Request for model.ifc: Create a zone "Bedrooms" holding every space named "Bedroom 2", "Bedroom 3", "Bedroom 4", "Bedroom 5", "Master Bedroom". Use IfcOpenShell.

First a look at what the model holds.

```python
import ifcopenshell

model = ifcopenshell.open("model.ifc")
print(model.schema)
seen = {}
for space in model.by_type("IfcSpace"):
    seen[space.LongName] = seen.get(space.LongName, 0) + 1
for name, count in sorted(seen.items(), key=str):
    print(count, "x", name)
print("zones:", [z.Name for z in model.by_type("IfcZone")][:20])
```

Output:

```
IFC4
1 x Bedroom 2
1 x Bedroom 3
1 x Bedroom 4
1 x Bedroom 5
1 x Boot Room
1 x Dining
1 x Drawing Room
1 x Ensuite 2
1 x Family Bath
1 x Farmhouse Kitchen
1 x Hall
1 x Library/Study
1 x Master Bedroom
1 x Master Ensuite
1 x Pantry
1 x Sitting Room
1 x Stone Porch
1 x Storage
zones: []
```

```python
import ifcopenshell
import ifcopenshell.api.group
import ifcopenshell.api.root

model = ifcopenshell.open("model.ifc")

names = {"Bedroom 2", "Bedroom 3", "Bedroom 4", "Bedroom 5", "Master Bedroom"}
spaces = [s for s in model.by_type("IfcSpace") if s.LongName in names]

zone = ifcopenshell.api.root.create_entity(model, ifc_class="IfcZone", name="Bedrooms")
ifcopenshell.api.group.assign_group(model, products=spaces, group=zone)
print(len(spaces), "spaces in", zone.Name)

model.write("model_updated.ifc")
```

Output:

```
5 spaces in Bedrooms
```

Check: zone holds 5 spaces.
